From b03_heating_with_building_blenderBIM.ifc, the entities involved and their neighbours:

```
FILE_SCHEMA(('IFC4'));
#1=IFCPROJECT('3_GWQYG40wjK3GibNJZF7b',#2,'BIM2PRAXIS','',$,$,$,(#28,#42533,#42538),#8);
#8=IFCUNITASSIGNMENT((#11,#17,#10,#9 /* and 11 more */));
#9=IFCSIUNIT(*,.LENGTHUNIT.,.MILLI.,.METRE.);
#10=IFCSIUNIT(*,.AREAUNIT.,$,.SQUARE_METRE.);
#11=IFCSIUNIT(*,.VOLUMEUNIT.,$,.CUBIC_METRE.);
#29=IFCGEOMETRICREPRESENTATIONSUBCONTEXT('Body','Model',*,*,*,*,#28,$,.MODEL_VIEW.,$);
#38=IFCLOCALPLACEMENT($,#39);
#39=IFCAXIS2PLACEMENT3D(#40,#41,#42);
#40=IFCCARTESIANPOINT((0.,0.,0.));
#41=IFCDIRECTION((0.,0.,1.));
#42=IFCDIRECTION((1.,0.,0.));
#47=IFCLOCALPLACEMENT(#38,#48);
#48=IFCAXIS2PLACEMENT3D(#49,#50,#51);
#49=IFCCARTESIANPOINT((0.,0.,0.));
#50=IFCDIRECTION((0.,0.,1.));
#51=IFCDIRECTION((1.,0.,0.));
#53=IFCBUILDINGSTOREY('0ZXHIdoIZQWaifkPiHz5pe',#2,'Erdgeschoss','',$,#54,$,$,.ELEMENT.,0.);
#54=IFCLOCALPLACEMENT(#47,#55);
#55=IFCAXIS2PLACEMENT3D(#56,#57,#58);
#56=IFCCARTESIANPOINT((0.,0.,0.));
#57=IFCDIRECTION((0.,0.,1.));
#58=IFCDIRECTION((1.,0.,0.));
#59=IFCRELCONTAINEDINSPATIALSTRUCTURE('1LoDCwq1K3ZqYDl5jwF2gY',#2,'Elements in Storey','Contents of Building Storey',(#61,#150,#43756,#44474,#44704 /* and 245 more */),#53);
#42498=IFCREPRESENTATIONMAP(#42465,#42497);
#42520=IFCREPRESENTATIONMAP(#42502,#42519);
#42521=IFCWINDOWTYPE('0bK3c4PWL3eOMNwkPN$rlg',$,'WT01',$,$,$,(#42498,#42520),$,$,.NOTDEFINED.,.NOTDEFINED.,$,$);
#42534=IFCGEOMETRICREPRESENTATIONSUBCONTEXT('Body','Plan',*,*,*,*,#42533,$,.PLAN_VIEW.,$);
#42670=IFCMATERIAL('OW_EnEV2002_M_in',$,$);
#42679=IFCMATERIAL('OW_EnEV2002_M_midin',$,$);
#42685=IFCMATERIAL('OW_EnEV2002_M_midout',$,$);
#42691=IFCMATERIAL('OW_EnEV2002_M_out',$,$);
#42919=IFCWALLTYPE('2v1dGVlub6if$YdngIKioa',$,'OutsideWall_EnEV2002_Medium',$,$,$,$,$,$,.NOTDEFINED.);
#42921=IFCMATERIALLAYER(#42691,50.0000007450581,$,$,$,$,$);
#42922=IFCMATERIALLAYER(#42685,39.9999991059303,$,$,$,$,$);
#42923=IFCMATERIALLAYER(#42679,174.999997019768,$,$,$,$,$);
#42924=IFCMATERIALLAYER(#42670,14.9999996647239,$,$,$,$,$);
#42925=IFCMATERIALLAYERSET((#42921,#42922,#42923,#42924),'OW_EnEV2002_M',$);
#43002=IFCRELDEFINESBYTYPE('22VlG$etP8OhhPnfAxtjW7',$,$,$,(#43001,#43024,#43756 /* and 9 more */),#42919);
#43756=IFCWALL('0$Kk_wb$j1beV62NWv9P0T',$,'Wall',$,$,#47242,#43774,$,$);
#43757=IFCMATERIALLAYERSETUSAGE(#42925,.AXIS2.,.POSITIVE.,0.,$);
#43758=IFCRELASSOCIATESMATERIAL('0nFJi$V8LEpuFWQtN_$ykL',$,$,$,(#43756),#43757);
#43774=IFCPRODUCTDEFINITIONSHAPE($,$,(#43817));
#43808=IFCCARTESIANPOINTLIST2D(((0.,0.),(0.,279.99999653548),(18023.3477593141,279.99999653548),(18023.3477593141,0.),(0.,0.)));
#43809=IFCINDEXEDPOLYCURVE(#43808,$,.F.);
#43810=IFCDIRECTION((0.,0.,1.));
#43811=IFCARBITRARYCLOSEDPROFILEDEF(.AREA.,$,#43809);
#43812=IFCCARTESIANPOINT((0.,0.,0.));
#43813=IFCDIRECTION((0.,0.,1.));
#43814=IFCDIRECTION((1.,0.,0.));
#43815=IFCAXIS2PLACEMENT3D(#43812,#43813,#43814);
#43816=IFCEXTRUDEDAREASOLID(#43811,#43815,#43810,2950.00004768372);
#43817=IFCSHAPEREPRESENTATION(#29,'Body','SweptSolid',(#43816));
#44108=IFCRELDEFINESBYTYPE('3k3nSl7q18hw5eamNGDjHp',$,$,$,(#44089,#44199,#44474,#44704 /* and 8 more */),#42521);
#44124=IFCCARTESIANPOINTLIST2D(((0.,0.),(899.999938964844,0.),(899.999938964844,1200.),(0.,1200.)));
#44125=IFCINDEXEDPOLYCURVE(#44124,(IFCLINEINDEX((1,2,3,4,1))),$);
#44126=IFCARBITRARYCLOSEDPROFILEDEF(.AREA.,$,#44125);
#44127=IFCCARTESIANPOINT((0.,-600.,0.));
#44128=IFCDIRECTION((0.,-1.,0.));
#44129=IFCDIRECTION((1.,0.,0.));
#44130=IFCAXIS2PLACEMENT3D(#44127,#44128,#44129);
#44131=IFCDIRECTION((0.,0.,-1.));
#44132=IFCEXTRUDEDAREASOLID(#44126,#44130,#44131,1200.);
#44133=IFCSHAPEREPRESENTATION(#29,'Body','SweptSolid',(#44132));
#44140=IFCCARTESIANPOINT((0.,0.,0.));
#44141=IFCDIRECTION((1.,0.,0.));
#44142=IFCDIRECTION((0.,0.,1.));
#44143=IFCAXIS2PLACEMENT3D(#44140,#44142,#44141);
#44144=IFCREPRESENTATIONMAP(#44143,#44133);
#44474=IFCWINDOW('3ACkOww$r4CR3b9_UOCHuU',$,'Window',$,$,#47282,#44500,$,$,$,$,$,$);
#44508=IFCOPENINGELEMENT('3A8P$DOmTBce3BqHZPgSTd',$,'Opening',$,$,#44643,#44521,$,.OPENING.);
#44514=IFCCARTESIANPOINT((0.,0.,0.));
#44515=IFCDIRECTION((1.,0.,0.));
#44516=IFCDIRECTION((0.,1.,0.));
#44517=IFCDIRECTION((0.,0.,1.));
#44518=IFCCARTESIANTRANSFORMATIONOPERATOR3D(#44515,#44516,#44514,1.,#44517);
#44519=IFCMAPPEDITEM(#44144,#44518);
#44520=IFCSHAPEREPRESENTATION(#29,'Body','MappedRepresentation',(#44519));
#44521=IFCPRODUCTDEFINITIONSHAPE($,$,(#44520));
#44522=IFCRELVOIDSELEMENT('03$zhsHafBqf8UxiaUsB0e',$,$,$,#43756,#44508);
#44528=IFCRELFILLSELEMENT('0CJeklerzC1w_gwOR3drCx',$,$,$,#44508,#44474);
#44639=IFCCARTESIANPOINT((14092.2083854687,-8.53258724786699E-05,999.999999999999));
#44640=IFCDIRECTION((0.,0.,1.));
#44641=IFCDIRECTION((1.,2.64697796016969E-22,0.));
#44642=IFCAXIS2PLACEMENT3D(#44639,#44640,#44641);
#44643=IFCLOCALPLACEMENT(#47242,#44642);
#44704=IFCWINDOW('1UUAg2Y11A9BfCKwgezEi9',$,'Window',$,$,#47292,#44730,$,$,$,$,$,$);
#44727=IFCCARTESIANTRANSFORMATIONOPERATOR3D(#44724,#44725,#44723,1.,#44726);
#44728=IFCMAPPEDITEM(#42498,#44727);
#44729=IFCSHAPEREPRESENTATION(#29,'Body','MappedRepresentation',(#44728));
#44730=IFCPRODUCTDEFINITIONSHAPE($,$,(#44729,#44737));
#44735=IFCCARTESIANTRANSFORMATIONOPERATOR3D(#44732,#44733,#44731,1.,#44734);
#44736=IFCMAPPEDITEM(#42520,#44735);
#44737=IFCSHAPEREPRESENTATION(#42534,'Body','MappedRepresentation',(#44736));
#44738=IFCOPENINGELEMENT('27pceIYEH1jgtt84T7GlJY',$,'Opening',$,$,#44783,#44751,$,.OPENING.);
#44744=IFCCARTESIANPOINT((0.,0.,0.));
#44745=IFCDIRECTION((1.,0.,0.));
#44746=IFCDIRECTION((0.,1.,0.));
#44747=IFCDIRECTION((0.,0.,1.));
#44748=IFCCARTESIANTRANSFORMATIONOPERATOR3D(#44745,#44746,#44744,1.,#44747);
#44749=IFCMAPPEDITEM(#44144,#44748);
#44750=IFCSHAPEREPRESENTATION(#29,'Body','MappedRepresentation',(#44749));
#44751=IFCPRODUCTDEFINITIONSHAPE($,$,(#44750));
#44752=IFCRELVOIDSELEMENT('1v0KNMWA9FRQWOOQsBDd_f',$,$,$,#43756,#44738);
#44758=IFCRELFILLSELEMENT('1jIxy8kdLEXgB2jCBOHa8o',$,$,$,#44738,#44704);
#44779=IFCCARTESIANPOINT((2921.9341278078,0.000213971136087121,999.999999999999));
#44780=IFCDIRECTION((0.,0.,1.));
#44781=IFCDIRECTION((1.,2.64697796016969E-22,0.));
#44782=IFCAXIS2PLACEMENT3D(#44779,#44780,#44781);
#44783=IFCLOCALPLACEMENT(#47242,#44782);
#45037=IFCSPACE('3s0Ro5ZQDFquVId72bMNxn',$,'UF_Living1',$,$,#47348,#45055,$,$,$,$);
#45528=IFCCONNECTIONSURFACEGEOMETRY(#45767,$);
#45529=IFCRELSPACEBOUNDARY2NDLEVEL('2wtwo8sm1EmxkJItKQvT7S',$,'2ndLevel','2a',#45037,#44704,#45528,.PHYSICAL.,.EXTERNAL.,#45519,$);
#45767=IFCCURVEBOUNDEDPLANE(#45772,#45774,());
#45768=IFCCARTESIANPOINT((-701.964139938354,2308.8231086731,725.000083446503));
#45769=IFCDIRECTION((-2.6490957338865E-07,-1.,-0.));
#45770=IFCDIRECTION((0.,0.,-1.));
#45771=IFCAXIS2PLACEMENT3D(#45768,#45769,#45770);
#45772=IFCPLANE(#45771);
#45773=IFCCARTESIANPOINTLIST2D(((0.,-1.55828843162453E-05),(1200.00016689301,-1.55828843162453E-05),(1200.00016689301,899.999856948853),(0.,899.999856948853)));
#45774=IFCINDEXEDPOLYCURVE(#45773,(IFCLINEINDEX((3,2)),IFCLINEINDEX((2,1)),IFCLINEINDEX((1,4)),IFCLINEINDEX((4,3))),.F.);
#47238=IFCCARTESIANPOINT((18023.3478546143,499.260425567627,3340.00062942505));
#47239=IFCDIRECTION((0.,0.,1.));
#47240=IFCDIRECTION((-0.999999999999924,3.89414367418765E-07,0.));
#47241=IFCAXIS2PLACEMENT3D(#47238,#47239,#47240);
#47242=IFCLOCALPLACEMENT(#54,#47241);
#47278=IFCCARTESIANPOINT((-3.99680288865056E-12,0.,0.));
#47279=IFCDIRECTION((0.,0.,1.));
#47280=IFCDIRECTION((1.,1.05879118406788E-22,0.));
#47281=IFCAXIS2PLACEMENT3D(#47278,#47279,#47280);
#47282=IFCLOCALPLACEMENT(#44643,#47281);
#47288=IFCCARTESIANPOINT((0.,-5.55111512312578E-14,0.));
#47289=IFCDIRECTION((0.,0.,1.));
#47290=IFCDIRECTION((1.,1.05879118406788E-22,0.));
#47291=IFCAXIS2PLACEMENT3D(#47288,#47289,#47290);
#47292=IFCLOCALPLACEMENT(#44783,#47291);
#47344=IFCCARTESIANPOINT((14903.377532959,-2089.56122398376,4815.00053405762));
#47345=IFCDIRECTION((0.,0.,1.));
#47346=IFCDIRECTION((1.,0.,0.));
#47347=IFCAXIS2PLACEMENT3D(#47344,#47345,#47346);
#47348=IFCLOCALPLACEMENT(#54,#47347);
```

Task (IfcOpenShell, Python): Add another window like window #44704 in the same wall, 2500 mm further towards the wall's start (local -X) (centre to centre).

```python
import numpy as np
import ifcopenshell
import ifcopenshell.api.feature
import ifcopenshell.api.geometry
import ifcopenshell.api.root
import ifcopenshell.geom
import ifcopenshell.util.element
import ifcopenshell.util.placement
import ifcopenshell.util.shape

model = ifcopenshell.open("b03_heating_with_building_blenderBIM.ifc")
settings = ifcopenshell.geom.settings()


def volume(element):
    """Net volume in cubic metres, openings subtracted."""
    shape = ifcopenshell.geom.create_shape(settings, element)
    return ifcopenshell.util.shape.get_volume(shape.geometry)


window = model.by_guid("1UUAg2Y11A9BfCKwgezEi9")
opening = window.FillsVoids[0].RelatingOpeningElement
wall = opening.VoidsElements[0].RelatingBuildingElement
before = volume(wall)
shift = ifcopenshell.util.placement.get_local_placement(wall.ObjectPlacement)[:3, 0] * -2500.0

# copy_class copies the void relationship, type, container and properties, but no geometry.
new_opening = ifcopenshell.api.root.copy_class(model, product=opening)
new_opening.Representation = ifcopenshell.util.element.copy_deep(
    model, opening.Representation, exclude=["IfcGeometricRepresentationContext", "IfcRepresentationMap"]
)
new_window = ifcopenshell.api.root.copy_class(model, product=window)
new_window.Representation = ifcopenshell.util.element.copy_deep(
    model, window.Representation, exclude=["IfcGeometricRepresentationContext", "IfcRepresentationMap"]
)
ifcopenshell.api.feature.add_filling(model, opening=new_opening, element=new_window)

for old, new in ((opening, new_opening), (window, new_window)):
    matrix = ifcopenshell.util.placement.get_local_placement(old.ObjectPlacement)
    matrix[:3, 3] += shift
    ifcopenshell.api.geometry.edit_object_placement(model, product=new, matrix=matrix, is_si=False)

# The copied space boundaries still share their surfaces with the original.
for rel in new_window.ProvidesBoundaries:
    if rel.ConnectionGeometry:
        rel.ConnectionGeometry = ifcopenshell.util.element.copy_deep(model, rel.ConnectionGeometry)

# Space boundary surfaces are stored in each space's coordinates; move them too.
for rel in new_window.ProvidesBoundaries:
    if not rel.ConnectionGeometry:
        continue
    surface = rel.ConnectionGeometry.SurfaceOnRelatingElement.BasisSurface
    space_matrix = ifcopenshell.util.placement.get_local_placement(rel.RelatingSpace.ObjectPlacement)
    point = np.array(surface.Position.Location.Coordinates) + space_matrix[:3, :3].T @ shift
    surface.Position = model.createIfcAxis2Placement3D(
        model.createIfcCartesianPoint(point.tolist()), surface.Position.Axis, surface.Position.RefDirection
    )

after = volume(wall)

print(f"wall volume {before:.3f} -> {after:.3f} m3")

model.write("b03_heating_with_building_blenderBIM_updated.ifc")
```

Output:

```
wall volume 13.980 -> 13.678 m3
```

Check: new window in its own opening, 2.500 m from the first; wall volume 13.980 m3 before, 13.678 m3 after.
